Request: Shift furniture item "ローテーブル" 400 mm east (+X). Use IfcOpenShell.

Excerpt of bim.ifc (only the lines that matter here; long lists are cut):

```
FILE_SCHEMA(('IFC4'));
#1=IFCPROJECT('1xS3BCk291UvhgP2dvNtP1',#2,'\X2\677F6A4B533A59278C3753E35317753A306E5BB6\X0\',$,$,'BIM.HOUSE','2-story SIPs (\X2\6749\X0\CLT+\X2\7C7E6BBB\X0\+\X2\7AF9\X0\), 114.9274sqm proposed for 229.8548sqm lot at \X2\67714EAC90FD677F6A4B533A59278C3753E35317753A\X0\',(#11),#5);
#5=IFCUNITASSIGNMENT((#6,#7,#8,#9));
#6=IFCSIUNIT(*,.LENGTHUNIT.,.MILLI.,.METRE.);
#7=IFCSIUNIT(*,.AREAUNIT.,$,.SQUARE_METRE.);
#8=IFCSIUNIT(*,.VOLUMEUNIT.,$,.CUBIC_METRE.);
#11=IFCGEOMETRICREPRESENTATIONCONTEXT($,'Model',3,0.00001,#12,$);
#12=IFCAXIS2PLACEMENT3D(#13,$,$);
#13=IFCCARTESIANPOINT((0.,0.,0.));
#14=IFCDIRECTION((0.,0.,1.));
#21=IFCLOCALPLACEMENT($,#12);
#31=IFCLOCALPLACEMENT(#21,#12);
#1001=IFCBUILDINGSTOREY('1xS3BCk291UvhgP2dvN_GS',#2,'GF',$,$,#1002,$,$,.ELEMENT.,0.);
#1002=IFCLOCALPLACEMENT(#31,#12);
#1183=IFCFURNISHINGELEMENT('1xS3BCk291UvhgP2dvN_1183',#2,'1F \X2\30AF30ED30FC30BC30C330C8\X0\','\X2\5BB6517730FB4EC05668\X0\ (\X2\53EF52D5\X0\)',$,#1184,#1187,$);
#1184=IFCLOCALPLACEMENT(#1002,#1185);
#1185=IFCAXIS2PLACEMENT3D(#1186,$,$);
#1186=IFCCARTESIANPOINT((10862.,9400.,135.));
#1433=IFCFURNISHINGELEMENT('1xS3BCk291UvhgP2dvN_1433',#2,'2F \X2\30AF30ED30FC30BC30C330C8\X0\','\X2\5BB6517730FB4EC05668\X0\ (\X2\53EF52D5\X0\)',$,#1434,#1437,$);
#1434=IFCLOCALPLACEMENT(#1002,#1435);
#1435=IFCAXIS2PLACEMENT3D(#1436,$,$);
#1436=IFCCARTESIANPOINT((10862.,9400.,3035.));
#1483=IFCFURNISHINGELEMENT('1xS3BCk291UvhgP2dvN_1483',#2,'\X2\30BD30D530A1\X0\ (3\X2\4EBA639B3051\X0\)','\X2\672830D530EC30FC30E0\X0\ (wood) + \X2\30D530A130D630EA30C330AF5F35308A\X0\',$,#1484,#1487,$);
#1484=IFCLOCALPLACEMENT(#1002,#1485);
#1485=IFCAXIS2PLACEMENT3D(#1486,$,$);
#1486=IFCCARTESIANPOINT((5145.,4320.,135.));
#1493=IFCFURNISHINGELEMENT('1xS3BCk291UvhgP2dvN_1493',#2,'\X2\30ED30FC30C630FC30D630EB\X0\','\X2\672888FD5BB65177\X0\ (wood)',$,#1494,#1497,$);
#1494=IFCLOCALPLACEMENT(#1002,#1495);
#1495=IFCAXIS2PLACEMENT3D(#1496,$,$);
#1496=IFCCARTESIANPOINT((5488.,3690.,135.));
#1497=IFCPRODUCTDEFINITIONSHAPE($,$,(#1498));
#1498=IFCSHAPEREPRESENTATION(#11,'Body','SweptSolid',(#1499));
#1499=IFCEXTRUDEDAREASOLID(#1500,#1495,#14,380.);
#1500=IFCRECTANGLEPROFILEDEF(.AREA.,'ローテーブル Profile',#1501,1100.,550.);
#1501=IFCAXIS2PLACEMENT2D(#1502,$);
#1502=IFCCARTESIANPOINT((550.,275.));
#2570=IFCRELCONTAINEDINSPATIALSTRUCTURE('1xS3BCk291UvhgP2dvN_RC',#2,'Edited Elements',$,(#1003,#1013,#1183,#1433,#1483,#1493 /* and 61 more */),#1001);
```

```python
import ifcopenshell
import ifcopenshell.api.geometry
import ifcopenshell.util.placement
import ifcopenshell.util.unit

model = ifcopenshell.open("bim.ifc")
unit_scale = ifcopenshell.util.unit.calculate_unit_scale(model)

item = model.by_guid("1xS3BCk291UvhgP2dvN_1493")
matrix = ifcopenshell.util.placement.get_local_placement(item.ObjectPlacement)
matrix[0, 3] += 0.4 / unit_scale
ifcopenshell.api.geometry.edit_object_placement(model, product=item, matrix=matrix, is_si=False)

print(ifcopenshell.util.placement.get_local_placement(item.ObjectPlacement).round(3) + 0.0)

model.write("bim_rev.ifc")
```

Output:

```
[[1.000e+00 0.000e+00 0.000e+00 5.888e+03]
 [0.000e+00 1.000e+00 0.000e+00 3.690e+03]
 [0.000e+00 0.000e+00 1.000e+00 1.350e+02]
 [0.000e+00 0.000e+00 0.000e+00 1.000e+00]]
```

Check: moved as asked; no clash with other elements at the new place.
